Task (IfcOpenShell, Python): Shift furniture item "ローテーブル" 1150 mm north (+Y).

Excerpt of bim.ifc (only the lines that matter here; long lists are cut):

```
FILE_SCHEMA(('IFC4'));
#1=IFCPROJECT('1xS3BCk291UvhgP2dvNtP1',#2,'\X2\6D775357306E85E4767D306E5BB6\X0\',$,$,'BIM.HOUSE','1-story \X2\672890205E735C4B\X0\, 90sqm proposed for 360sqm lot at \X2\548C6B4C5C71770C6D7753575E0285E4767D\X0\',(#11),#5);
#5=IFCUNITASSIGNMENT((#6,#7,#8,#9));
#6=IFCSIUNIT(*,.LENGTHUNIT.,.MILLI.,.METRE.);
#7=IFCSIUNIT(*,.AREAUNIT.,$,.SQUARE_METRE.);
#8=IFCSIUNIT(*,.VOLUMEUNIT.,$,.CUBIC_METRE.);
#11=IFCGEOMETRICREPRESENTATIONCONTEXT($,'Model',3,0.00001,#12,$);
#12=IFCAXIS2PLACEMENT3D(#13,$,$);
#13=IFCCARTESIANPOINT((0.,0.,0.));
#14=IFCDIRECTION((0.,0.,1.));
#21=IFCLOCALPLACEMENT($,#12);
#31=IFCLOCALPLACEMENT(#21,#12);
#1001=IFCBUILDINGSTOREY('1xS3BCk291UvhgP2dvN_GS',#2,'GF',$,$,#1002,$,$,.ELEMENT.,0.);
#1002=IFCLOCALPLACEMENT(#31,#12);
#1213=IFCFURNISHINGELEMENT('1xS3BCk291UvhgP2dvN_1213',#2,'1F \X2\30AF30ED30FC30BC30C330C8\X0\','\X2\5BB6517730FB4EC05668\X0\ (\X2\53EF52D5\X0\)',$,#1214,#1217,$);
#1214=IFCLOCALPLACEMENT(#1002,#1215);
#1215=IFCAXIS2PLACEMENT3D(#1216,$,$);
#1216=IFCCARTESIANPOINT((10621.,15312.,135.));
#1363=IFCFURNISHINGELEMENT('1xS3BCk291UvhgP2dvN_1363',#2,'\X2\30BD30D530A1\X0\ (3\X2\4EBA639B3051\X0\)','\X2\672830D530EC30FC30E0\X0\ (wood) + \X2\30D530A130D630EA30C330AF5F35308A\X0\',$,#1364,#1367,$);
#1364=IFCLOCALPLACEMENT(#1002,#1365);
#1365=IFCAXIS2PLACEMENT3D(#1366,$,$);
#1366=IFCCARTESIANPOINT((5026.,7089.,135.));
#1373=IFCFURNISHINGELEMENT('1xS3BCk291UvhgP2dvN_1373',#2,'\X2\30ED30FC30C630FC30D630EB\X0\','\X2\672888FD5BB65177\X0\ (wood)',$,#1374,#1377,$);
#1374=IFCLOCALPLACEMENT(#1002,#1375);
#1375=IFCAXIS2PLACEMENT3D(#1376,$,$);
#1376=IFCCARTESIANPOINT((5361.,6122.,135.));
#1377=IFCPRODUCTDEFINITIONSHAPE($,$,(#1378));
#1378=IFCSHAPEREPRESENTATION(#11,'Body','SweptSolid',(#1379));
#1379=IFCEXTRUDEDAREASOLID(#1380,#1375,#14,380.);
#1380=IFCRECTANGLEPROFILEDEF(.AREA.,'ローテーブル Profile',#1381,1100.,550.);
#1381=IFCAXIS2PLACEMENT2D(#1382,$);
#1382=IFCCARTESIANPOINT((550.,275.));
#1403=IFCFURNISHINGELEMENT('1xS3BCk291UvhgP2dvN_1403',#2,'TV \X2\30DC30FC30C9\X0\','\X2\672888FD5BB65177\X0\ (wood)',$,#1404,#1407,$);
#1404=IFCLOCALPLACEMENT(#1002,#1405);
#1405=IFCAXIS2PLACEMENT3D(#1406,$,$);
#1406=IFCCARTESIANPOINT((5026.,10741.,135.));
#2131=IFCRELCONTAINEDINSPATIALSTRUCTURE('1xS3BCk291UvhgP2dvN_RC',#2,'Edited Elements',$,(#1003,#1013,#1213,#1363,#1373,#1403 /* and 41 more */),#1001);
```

```python
import ifcopenshell
import ifcopenshell.api.geometry
import ifcopenshell.util.placement
import ifcopenshell.util.unit

model = ifcopenshell.open("bim.ifc")
unit_scale = ifcopenshell.util.unit.calculate_unit_scale(model)

item = model.by_id(1373)
matrix = ifcopenshell.util.placement.get_local_placement(item.ObjectPlacement)
matrix[1, 3] += 1.15 / unit_scale
ifcopenshell.api.geometry.edit_object_placement(model, product=item, matrix=matrix, is_si=False)

print(ifcopenshell.util.placement.get_local_placement(item.ObjectPlacement).round(3) + 0.0)

model.write("bim-out.ifc")
```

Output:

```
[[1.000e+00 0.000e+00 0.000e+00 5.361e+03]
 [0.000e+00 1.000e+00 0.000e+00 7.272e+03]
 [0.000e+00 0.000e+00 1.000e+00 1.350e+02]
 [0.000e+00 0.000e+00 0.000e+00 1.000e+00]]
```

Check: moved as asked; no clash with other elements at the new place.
